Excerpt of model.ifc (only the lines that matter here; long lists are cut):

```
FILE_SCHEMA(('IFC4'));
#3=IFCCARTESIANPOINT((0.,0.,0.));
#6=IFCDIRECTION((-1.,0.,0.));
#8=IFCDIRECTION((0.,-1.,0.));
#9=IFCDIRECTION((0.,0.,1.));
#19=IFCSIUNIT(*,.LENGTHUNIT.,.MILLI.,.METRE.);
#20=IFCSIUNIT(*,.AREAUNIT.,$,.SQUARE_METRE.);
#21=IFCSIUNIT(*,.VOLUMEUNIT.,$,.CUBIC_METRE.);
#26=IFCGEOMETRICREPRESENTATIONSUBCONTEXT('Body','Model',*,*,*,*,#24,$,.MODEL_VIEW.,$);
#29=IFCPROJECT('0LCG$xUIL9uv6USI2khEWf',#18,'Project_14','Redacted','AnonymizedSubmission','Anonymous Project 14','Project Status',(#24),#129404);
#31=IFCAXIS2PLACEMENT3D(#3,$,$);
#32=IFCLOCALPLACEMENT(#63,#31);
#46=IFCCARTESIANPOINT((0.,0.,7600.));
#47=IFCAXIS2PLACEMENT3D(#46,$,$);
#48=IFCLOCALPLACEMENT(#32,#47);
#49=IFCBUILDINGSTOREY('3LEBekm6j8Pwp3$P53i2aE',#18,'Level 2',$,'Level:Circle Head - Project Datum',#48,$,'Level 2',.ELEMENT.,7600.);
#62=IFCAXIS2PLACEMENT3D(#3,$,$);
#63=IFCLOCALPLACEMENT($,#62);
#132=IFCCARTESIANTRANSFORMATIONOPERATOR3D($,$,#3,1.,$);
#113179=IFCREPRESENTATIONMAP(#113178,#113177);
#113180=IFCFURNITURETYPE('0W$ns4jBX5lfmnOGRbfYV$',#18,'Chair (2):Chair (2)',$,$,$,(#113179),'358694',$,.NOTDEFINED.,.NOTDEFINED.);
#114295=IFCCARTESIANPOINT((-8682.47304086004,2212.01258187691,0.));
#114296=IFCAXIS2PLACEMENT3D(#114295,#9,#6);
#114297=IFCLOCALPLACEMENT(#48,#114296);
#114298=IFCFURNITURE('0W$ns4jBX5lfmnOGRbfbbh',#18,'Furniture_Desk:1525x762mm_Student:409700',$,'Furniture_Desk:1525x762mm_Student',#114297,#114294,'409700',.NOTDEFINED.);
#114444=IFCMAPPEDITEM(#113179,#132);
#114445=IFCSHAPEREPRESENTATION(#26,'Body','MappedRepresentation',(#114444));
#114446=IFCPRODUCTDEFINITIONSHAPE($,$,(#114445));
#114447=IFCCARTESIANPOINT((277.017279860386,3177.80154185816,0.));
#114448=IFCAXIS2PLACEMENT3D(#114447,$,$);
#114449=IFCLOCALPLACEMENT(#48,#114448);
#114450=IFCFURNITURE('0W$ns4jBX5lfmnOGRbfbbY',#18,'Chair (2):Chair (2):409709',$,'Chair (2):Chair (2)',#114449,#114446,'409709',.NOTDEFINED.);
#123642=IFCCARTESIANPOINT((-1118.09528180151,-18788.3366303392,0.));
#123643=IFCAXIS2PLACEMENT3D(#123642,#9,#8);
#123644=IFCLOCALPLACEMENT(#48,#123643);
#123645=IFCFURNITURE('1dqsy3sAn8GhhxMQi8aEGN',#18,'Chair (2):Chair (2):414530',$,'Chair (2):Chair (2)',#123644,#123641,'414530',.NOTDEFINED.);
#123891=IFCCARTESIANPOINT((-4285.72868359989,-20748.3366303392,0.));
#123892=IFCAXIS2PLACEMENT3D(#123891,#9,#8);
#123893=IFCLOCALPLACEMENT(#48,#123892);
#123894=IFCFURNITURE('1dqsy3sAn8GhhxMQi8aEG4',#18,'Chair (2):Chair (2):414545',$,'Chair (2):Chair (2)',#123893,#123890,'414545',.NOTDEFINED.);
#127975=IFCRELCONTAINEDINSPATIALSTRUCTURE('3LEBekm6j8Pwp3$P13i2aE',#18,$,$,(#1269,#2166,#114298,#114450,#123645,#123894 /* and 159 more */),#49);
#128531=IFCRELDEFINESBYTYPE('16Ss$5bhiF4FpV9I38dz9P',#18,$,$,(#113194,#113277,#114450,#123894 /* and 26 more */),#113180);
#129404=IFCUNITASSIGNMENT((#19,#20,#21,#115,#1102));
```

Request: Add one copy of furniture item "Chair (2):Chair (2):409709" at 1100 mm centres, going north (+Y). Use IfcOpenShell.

```python
import numpy as np
import ifcopenshell
import ifcopenshell.api.geometry
import ifcopenshell.api.root
import ifcopenshell.util.element
import ifcopenshell.util.placement
import ifcopenshell.util.unit

model = ifcopenshell.open("model.ifc")
unit_scale = ifcopenshell.util.unit.calculate_unit_scale(model)


def reuse_history(source, copy):
    """copy_class also copies each property set's owner history, people and application; keep the originals."""
    for rel in copy.IsDefinedBy:
        if rel.is_a("IfcRelDefinesByProperties") and (history := rel.RelatingPropertyDefinition.OwnerHistory):
            rel.RelatingPropertyDefinition.OwnerHistory = source.OwnerHistory
            ifcopenshell.util.element.remove_deep2(model, history)


source = model.by_guid("0W$ns4jBX5lfmnOGRbfbbY")
base = ifcopenshell.util.placement.get_local_placement(source.ObjectPlacement)
step = np.array([0.0, 1.0, 0.0]) * 1.1 / unit_scale

for i in range(1, 2):
    copy = ifcopenshell.api.root.copy_class(model, product=source)
    copy.Representation = ifcopenshell.util.element.copy_deep(
        model, source.Representation, exclude=["IfcGeometricRepresentationContext", "IfcRepresentationMap"]
    )
    copy.Name = "Chair (2):Chair (2)"
    copy.Tag = None
    reuse_history(source, copy)
    matrix = base.copy()
    matrix[:3, 3] += i * step
    print("added at", matrix[:3, 3].round(3) + 0.0)
    ifcopenshell.api.geometry.edit_object_placement(model, product=copy, matrix=matrix, is_si=False)

model.write("model_updated.ifc")
```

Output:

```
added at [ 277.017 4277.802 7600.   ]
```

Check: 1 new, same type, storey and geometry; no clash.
